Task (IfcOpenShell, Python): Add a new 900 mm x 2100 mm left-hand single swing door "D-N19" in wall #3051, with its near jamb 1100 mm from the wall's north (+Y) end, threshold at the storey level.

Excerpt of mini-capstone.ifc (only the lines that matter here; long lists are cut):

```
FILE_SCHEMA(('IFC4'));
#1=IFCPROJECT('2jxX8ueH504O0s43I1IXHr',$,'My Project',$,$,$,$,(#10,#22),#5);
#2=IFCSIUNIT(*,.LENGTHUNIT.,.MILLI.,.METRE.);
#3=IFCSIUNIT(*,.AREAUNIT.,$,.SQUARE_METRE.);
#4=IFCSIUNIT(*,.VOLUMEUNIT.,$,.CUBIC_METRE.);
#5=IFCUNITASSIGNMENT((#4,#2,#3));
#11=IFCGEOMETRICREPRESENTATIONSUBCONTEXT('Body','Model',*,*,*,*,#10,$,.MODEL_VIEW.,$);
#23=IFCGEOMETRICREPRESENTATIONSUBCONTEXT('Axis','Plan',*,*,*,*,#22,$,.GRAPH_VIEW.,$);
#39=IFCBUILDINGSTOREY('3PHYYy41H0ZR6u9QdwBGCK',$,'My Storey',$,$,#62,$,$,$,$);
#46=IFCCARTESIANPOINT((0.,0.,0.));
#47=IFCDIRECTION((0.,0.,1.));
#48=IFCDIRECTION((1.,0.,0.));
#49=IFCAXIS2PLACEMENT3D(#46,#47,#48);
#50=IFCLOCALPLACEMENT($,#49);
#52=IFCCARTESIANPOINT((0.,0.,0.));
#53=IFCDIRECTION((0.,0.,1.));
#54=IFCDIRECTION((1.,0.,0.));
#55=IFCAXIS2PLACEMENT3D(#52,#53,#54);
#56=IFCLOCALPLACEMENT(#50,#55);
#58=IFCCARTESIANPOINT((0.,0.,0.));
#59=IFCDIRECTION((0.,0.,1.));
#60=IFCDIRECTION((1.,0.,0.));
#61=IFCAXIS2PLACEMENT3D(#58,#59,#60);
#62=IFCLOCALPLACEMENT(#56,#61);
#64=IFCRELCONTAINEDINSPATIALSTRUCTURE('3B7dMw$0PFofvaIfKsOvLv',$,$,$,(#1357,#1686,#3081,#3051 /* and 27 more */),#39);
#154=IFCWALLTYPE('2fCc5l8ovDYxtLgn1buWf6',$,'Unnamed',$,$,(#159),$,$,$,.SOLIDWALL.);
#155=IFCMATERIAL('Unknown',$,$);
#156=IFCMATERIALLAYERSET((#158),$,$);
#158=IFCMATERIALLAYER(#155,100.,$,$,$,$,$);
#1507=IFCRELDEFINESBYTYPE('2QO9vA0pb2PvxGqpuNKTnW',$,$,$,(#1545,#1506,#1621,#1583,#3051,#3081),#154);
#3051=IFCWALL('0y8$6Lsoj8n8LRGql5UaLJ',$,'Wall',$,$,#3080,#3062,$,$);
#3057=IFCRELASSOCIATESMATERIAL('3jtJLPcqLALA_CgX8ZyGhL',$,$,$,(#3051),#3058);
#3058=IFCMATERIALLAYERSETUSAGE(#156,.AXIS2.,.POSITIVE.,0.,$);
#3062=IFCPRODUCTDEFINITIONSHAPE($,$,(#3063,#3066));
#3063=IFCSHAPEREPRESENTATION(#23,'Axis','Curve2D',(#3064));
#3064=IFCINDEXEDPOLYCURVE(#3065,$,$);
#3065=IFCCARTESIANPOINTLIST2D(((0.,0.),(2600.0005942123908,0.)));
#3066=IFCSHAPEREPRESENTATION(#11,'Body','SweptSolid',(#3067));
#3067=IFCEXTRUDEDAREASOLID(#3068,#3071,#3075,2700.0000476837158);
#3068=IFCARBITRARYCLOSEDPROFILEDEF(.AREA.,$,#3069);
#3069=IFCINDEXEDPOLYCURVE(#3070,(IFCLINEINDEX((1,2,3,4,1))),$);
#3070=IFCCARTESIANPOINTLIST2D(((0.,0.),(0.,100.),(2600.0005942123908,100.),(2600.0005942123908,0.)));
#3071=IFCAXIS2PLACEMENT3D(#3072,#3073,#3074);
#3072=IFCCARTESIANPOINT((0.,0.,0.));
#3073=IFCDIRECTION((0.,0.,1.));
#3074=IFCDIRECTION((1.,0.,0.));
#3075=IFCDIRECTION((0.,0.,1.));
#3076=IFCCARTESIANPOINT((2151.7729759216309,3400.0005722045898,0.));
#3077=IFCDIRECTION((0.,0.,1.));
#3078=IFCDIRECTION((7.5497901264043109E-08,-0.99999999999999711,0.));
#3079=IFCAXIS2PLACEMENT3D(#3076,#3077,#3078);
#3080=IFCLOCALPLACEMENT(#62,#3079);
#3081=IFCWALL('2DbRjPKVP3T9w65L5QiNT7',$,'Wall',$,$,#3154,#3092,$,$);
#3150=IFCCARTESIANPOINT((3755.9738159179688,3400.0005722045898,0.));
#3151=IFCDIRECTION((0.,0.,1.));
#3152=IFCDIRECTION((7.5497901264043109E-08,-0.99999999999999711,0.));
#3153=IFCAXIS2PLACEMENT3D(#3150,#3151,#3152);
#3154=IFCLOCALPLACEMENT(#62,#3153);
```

```python
import numpy as np
import ifcopenshell
import ifcopenshell.api.feature
import ifcopenshell.api.geometry
import ifcopenshell.api.root
import ifcopenshell.api.spatial
import ifcopenshell.geom
import ifcopenshell.util.element
import ifcopenshell.util.placement
import ifcopenshell.util.representation
import ifcopenshell.util.shape
import ifcopenshell.util.unit

model = ifcopenshell.open("mini-capstone.ifc")
unit_scale = ifcopenshell.util.unit.calculate_unit_scale(model)
settings = ifcopenshell.geom.settings()


def volume(element):
    """Net volume in cubic metres, openings subtracted."""
    shape = ifcopenshell.geom.create_shape(settings, element)
    return ifcopenshell.util.shape.get_volume(shape.geometry)


wall = model.by_guid("0y8$6Lsoj8n8LRGql5UaLJ")
storey = ifcopenshell.util.element.get_container(wall, ifc_class="IfcBuildingStorey")
context = ifcopenshell.util.representation.get_context(model, "Model", "Body", "MODEL_VIEW")
before = volume(wall)

width, height, from_end, sill = 0.9, 2.1, 1.1, 0.0  # metres

# The wall runs along its own X axis, and the end named is its -X end.
wall_shape = ifcopenshell.geom.create_shape(settings, wall)
x, y, z = ifcopenshell.util.shape.get_vertices(wall_shape.geometry).T
start = x.min() + from_end
face, thickness = float(y.min()), float(y.max() - y.min())
wall_matrix = ifcopenshell.util.placement.get_local_placement(wall.ObjectPlacement)
level = ifcopenshell.util.placement.get_local_placement(storey.ObjectPlacement)[2, 3]


def in_wall(x, y):
    """Placement at x, y metres in the wall's axes, at sill height."""
    matrix = wall_matrix.copy()
    matrix[:, 3] = wall_matrix @ np.array([x / unit_scale, y / unit_scale, 0.0, 1.0])
    matrix[2, 3] = level + sill / unit_scale
    return matrix


# Opening: a box that overshoots both wall faces by 50 mm.
opening = ifcopenshell.api.root.create_entity(model, ifc_class="IfcOpeningElement", predefined_type="OPENING")
box = ifcopenshell.api.geometry.add_wall_representation(
    model, context=context, length=width, height=height, thickness=thickness + 0.1
)
ifcopenshell.api.geometry.assign_representation(model, product=opening, representation=box)
ifcopenshell.api.geometry.edit_object_placement(model, product=opening, matrix=in_wall(start, face - 0.05), is_si=False)
ifcopenshell.api.feature.add_feature(model, feature=opening, element=wall)

door = ifcopenshell.api.root.create_entity(model, ifc_class="IfcDoor", name="D-N19", predefined_type="DOOR")
door.OverallWidth, door.OverallHeight = width / unit_scale, height / unit_scale
door.OperationType = "SINGLE_SWING_LEFT"
body = ifcopenshell.api.geometry.add_door_representation(
    model,
    context=context,
    overall_width=door.OverallWidth,
    overall_height=door.OverallHeight,
    operation_type="SINGLE_SWING_LEFT",
    lining_properties={"LiningDepth": thickness / unit_scale, "ThresholdDepth": thickness / unit_scale},
)
ifcopenshell.api.geometry.assign_representation(model, product=door, representation=body)
ifcopenshell.api.spatial.assign_container(model, products=[door], relating_structure=storey)
ifcopenshell.api.feature.add_filling(model, opening=opening, element=door)

# The lining spans the wall, so the door starts at the wall face.
ifcopenshell.api.geometry.edit_object_placement(model, product=door, matrix=in_wall(start, face), is_si=False)

after = volume(wall)

print(f"wall volume {before:.3f} -> {after:.3f} m3")

model.write("mini-capstone_edited.ifc")
```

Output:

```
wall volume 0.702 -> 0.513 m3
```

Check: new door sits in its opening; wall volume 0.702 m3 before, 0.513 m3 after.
